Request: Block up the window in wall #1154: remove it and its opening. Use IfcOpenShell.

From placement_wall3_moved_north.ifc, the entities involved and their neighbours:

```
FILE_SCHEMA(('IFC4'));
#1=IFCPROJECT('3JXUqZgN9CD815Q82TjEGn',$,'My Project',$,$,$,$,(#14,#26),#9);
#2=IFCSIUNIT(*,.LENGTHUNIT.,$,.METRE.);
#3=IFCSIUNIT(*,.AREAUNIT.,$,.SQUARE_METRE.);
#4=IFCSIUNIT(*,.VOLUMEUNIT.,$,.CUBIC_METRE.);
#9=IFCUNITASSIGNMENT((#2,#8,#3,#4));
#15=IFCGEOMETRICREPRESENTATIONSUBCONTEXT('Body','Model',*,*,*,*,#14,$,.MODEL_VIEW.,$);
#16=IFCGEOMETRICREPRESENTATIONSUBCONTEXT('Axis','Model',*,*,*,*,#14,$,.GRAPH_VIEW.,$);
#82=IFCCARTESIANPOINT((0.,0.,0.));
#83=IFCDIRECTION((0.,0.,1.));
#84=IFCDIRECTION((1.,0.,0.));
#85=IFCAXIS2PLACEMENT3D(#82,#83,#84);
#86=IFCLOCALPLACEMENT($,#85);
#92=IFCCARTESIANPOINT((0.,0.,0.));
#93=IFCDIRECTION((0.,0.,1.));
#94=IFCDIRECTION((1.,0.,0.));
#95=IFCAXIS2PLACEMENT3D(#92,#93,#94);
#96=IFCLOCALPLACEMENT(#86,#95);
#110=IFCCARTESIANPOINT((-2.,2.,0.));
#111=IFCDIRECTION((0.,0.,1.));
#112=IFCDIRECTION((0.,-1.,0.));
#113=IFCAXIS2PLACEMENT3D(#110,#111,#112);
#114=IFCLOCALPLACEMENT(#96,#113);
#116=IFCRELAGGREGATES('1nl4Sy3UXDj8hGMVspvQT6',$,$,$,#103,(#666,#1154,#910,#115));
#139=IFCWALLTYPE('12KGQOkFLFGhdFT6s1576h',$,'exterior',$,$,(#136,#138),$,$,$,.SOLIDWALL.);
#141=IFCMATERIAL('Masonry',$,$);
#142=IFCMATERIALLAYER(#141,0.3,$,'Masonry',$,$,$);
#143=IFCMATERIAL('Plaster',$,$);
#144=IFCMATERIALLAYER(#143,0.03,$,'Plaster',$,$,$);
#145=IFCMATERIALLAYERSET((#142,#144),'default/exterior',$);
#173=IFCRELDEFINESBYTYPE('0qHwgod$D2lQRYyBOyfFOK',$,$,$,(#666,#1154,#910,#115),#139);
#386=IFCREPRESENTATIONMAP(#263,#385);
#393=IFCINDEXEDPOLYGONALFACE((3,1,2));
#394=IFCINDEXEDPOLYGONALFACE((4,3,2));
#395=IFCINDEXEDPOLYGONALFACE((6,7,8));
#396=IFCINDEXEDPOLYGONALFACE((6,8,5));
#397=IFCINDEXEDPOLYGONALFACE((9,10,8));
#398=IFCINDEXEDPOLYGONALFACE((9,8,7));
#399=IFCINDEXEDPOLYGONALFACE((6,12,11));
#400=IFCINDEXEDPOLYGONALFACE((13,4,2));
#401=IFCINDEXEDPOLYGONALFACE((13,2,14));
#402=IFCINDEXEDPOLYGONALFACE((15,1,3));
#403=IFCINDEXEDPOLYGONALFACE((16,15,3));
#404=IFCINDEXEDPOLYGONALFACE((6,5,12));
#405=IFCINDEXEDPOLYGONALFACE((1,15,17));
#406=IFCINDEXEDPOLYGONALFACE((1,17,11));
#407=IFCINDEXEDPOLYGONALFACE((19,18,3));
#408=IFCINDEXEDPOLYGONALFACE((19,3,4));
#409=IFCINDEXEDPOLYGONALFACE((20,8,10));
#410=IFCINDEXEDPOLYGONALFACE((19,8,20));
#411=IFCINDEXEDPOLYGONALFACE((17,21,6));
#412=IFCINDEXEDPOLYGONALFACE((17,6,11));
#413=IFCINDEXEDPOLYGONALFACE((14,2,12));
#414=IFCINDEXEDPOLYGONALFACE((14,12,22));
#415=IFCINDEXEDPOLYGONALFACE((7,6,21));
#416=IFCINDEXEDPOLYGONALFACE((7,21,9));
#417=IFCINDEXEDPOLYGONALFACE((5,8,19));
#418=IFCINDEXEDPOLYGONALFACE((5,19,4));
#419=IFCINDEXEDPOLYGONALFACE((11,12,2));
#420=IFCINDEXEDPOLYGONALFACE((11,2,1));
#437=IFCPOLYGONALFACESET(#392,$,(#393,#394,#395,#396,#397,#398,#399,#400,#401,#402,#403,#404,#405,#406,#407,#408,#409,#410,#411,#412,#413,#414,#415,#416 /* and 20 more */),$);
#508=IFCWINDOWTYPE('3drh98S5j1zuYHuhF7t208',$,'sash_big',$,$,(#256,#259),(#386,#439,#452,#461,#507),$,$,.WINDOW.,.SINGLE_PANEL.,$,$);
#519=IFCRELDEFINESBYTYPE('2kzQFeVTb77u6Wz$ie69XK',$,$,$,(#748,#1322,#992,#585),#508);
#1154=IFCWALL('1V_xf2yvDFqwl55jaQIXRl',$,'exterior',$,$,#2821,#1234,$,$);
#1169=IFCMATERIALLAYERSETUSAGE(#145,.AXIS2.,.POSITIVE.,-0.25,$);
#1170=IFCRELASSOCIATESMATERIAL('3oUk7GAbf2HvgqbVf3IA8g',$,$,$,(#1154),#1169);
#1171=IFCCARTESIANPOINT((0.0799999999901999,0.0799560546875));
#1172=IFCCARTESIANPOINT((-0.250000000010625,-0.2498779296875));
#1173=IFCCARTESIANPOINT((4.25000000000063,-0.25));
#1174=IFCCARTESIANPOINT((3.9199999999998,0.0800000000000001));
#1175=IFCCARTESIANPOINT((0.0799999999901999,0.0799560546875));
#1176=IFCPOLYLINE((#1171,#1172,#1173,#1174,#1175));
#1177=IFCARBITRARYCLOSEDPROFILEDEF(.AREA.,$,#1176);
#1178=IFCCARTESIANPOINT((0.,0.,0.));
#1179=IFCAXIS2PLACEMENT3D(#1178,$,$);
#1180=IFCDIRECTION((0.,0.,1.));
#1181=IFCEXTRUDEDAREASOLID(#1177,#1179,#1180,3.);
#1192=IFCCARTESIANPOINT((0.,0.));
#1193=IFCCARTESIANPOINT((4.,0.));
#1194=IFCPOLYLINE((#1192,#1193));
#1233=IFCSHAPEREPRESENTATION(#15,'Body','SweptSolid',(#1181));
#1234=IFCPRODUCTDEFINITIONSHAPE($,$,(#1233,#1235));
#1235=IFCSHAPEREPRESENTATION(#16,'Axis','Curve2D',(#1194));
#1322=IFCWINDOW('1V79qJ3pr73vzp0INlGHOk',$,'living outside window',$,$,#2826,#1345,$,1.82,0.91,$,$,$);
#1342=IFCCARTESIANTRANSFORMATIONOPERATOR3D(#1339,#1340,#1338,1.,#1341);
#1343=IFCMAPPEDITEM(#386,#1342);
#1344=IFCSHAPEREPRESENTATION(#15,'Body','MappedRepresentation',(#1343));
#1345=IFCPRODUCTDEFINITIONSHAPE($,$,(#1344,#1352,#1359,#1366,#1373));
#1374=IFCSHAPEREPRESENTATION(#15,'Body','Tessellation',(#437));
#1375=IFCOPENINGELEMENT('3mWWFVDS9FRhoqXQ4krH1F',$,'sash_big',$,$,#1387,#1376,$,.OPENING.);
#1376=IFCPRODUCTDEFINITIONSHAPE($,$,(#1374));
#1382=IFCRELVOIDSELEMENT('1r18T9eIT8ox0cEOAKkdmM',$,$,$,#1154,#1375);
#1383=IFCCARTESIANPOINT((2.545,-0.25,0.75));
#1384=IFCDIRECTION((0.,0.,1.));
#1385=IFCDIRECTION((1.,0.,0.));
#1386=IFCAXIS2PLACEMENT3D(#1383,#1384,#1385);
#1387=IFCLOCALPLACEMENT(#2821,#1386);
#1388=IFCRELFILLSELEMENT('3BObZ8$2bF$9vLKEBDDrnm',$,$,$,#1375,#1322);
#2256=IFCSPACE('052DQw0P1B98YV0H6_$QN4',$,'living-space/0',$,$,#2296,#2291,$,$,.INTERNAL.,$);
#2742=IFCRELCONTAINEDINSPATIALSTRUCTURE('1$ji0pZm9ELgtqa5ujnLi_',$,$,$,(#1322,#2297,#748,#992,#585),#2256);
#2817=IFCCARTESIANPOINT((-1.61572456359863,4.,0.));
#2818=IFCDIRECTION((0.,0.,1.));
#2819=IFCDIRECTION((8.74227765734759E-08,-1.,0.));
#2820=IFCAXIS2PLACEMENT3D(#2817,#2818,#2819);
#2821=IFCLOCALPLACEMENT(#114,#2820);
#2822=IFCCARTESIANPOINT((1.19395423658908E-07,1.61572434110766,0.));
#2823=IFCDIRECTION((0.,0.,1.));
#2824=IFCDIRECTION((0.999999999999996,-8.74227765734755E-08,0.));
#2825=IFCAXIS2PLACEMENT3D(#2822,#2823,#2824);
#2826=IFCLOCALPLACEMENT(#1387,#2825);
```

```python
import ifcopenshell
import ifcopenshell.api.feature
import ifcopenshell.api.root
import ifcopenshell.geom
import ifcopenshell.util.shape

model = ifcopenshell.open("placement_wall3_moved_north.ifc")
settings = ifcopenshell.geom.settings()


def volume(element):
    """Net volume in cubic metres, openings subtracted."""
    shape = ifcopenshell.geom.create_shape(settings, element)
    return ifcopenshell.util.shape.get_volume(shape.geometry)


window = model.by_guid("1V79qJ3pr73vzp0INlGHOk")
opening = window.FillsVoids[0].RelatingOpeningElement
wall = opening.VoidsElements[0].RelatingBuildingElement
before = volume(wall)

ifcopenshell.api.root.remove_product(model, product=window)
ifcopenshell.api.feature.remove_feature(model, feature=opening)

after = volume(wall)

print(f"wall volume {before:.3f} -> {after:.3f} m3")

model.write("placement_wall3_moved_north_edited.ifc")
```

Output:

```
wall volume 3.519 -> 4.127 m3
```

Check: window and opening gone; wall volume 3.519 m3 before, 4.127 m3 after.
